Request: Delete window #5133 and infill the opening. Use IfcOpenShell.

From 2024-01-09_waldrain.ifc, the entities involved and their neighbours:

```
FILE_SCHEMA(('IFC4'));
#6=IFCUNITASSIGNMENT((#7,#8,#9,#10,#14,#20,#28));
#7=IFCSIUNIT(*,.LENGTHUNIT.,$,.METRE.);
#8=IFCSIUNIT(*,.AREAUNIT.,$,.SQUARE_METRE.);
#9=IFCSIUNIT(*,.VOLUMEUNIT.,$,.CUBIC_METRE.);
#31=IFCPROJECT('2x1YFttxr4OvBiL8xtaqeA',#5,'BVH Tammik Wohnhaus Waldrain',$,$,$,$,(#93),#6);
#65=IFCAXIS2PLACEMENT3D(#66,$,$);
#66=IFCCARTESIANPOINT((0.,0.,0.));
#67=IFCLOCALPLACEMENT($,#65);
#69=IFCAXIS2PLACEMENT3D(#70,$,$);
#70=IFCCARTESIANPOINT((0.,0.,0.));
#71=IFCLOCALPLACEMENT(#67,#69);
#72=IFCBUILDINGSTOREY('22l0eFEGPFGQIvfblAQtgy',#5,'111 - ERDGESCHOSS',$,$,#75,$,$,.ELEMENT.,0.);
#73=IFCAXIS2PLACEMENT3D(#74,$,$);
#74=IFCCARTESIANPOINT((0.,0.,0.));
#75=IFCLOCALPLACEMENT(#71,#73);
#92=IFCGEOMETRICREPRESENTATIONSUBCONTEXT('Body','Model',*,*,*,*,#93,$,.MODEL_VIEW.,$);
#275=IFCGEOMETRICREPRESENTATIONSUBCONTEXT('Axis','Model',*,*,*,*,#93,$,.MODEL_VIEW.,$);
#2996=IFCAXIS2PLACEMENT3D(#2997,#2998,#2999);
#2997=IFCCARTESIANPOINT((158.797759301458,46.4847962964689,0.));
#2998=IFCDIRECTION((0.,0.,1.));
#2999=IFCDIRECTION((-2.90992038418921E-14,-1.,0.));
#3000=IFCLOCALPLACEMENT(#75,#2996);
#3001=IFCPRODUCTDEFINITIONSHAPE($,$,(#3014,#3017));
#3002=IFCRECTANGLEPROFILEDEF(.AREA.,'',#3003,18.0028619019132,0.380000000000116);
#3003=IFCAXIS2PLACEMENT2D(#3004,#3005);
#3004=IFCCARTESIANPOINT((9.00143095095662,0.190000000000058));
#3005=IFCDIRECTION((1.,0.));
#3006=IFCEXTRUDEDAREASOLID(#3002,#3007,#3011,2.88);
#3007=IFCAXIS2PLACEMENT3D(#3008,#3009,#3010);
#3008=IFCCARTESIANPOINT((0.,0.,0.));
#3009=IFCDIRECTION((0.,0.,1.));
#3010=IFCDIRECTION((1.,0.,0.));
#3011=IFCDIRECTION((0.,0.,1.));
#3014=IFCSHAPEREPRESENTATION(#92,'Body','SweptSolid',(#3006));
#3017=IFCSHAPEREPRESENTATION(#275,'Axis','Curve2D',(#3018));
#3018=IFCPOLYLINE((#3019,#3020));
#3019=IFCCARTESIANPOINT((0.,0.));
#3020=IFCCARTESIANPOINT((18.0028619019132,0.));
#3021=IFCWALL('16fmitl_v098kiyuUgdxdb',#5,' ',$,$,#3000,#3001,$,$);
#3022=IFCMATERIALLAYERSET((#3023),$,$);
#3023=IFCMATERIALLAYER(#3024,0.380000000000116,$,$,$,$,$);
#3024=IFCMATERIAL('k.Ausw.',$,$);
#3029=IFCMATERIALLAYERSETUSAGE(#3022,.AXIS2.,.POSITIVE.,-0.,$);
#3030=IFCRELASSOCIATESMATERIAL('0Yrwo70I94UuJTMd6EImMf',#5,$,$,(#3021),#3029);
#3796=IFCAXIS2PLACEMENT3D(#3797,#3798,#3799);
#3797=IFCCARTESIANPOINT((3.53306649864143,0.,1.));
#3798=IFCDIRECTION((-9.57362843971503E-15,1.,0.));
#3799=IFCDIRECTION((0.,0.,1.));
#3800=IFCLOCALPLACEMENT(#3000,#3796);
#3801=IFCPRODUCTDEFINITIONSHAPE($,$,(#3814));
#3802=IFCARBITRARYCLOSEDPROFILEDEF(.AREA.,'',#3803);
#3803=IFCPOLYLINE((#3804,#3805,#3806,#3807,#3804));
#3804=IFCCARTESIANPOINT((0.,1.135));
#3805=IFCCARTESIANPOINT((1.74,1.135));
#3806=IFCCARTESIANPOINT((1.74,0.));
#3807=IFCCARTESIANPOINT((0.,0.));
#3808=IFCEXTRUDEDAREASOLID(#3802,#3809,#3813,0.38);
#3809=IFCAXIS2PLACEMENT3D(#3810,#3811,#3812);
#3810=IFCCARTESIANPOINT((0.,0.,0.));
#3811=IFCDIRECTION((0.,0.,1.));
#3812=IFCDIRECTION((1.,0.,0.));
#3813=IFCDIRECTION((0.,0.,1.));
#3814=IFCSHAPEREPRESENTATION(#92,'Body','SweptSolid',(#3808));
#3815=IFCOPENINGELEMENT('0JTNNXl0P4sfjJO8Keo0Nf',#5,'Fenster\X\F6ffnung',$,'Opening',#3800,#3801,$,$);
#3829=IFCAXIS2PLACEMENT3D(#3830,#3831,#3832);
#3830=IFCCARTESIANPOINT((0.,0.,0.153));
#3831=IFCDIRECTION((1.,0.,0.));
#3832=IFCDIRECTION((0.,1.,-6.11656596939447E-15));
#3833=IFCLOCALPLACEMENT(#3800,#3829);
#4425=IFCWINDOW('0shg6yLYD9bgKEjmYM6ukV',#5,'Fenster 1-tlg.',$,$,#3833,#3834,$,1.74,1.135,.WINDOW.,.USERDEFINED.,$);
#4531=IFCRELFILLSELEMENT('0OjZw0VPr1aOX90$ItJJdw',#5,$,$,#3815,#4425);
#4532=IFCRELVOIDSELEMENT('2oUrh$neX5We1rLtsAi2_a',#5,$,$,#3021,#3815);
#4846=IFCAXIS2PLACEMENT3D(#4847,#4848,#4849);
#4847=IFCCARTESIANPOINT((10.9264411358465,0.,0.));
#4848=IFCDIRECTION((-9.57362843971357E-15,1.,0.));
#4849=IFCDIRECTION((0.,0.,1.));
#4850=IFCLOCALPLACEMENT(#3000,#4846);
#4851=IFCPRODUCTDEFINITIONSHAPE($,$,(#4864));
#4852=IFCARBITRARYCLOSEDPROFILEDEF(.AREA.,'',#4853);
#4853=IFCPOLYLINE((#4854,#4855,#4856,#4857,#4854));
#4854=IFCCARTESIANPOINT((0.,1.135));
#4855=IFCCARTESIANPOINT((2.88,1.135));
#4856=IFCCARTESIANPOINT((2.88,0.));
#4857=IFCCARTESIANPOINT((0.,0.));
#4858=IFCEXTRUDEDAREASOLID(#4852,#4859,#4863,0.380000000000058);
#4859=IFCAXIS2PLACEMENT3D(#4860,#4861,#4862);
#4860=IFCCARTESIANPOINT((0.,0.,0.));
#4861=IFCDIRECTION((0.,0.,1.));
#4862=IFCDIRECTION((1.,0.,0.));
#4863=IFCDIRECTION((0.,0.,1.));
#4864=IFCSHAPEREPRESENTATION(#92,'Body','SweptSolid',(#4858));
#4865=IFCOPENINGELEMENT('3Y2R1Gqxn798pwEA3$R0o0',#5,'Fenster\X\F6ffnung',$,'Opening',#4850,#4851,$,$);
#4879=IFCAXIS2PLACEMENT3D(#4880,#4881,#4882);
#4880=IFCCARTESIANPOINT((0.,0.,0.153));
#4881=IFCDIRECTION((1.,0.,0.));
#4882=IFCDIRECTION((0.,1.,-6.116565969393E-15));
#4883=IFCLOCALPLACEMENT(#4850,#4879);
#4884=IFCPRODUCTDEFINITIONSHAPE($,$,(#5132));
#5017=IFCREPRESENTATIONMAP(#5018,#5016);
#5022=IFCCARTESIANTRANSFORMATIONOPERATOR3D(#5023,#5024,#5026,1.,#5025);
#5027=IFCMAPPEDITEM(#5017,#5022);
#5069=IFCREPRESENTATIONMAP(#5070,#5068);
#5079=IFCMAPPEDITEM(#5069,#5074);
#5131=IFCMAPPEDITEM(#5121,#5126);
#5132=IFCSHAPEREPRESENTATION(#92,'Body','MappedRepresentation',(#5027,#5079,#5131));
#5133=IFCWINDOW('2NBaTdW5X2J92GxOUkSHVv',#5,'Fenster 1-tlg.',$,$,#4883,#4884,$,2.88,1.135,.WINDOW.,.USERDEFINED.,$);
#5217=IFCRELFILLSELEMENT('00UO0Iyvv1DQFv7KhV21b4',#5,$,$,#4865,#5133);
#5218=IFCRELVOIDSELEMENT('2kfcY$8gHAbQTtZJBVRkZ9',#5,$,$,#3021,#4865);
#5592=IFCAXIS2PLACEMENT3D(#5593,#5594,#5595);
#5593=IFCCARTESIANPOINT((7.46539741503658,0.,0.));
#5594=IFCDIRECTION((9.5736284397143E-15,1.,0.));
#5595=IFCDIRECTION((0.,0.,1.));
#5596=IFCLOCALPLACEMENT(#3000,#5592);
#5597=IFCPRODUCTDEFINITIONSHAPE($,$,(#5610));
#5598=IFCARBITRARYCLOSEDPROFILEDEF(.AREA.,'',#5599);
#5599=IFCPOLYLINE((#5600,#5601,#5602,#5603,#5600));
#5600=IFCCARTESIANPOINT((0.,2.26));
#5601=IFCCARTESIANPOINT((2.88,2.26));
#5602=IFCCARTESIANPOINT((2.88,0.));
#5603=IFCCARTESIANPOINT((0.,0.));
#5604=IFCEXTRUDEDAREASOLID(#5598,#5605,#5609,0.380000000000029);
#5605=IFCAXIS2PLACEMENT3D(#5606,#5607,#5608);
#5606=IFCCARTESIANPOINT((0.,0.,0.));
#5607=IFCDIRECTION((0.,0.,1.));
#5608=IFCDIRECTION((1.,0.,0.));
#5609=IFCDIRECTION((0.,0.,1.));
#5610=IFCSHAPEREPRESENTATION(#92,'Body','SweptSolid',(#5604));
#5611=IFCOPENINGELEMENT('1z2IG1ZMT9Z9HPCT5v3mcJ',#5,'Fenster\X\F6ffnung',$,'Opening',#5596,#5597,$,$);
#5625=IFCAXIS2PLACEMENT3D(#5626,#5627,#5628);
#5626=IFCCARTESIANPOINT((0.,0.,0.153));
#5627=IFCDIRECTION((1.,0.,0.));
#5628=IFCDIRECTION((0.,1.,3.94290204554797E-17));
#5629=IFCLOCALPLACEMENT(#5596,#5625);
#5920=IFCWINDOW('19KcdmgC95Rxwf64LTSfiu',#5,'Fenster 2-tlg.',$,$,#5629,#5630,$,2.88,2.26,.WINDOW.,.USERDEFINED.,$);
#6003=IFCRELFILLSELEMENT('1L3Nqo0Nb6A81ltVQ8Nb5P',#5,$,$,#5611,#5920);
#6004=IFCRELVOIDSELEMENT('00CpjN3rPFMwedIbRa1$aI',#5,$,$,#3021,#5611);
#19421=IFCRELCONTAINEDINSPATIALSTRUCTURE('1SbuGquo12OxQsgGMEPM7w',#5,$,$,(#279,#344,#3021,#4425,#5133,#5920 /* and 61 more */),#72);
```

```python
import ifcopenshell
import ifcopenshell.api.feature
import ifcopenshell.api.root
import ifcopenshell.geom
import ifcopenshell.util.shape

model = ifcopenshell.open("2024-01-09_waldrain.ifc")
settings = ifcopenshell.geom.settings()


def volume(element):
    """Net volume in cubic metres, openings subtracted."""
    shape = ifcopenshell.geom.create_shape(settings, element)
    return ifcopenshell.util.shape.get_volume(shape.geometry)


window = model.by_guid("2NBaTdW5X2J92GxOUkSHVv")
opening = window.FillsVoids[0].RelatingOpeningElement
wall = opening.VoidsElements[0].RelatingBuildingElement
before = volume(wall)

ifcopenshell.api.root.remove_product(model, product=window)
ifcopenshell.api.feature.remove_feature(model, feature=opening)

after = volume(wall)

print(f"wall volume {before:.3f} -> {after:.3f} m3")

model.write("2024-01-09_waldrain_v2.ifc")
```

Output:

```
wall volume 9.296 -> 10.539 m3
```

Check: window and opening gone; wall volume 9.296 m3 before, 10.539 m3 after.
